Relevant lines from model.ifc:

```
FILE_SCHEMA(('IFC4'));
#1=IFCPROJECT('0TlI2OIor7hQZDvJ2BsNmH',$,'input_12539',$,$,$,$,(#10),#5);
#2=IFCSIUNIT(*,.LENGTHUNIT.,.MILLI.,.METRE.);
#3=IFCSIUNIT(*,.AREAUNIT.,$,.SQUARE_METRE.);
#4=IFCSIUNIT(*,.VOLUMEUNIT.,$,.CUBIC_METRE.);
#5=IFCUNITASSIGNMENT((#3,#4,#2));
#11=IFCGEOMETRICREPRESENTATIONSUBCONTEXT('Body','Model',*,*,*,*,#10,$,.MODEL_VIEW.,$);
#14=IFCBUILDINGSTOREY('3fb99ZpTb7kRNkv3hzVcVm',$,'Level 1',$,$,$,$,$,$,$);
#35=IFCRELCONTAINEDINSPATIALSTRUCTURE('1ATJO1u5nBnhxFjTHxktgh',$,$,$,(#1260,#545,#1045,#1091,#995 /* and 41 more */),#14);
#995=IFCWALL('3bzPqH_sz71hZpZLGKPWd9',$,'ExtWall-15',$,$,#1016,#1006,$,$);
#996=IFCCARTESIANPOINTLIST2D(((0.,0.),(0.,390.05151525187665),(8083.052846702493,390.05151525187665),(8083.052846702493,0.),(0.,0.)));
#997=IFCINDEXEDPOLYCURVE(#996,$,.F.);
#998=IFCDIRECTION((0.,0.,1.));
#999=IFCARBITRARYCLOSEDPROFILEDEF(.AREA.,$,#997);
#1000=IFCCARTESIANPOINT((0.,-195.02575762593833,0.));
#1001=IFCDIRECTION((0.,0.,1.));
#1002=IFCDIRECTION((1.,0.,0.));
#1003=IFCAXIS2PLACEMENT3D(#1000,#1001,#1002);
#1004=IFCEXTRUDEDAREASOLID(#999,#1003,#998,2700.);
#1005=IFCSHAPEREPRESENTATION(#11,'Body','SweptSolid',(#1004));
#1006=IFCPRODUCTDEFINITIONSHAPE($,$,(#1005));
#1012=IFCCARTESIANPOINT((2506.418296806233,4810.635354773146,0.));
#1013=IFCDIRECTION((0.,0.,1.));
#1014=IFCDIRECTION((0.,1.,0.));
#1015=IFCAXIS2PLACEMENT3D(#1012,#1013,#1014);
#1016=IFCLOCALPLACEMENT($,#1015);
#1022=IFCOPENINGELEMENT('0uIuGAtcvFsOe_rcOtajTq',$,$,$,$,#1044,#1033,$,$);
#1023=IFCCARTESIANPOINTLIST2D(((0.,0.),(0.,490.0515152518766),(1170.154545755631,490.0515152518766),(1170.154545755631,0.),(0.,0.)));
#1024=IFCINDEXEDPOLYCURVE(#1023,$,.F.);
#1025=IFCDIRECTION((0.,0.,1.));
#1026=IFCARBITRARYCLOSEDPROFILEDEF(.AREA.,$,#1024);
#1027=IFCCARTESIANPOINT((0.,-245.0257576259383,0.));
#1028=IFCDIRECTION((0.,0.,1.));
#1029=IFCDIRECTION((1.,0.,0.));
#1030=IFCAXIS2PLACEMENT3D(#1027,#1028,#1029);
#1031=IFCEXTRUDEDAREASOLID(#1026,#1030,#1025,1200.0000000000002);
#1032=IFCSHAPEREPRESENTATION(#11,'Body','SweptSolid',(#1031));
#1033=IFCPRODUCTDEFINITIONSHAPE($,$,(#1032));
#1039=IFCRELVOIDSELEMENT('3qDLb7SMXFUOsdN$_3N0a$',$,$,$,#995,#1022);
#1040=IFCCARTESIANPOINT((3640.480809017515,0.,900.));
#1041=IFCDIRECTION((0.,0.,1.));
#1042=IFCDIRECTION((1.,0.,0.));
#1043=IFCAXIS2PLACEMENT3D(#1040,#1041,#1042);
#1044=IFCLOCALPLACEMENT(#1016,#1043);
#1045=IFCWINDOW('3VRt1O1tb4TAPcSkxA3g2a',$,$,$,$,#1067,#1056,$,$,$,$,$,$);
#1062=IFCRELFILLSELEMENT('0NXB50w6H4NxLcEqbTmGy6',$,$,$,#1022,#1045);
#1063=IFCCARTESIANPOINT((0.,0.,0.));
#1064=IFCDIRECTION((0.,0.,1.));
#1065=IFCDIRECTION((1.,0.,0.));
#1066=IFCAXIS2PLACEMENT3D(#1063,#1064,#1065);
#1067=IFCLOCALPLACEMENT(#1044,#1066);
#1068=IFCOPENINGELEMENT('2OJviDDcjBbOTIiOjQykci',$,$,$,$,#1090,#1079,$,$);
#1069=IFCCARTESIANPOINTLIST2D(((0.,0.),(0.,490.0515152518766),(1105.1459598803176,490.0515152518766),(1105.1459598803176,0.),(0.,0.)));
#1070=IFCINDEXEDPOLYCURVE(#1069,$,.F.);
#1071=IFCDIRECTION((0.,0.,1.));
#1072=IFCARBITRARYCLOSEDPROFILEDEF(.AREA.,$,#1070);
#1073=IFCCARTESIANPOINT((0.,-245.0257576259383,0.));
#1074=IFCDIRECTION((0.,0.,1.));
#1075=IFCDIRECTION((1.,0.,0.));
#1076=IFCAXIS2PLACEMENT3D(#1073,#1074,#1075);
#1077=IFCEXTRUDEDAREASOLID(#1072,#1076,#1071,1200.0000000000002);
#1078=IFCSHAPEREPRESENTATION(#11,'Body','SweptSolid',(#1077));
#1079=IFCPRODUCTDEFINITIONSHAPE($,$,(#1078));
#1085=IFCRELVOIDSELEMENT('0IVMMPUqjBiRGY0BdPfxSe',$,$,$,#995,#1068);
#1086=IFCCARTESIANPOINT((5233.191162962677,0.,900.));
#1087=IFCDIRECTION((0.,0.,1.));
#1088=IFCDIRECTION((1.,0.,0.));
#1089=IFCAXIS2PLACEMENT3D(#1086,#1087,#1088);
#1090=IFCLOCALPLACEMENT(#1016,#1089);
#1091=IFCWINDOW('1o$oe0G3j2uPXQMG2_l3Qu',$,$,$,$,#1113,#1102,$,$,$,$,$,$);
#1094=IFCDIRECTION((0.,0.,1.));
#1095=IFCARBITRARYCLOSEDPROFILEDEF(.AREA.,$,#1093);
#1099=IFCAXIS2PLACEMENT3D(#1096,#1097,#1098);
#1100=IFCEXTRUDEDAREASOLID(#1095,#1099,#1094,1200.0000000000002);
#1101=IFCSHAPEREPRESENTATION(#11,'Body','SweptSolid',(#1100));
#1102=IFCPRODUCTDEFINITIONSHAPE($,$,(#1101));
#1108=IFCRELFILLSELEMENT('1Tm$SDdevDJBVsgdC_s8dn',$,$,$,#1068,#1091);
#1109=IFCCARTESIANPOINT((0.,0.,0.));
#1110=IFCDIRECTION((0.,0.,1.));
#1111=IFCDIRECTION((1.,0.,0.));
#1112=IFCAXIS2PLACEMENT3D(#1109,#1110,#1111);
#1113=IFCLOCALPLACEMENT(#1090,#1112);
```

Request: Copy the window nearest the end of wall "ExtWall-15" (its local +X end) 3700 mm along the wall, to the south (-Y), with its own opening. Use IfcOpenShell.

```python
import ifcopenshell
import ifcopenshell.api.feature
import ifcopenshell.api.geometry
import ifcopenshell.api.root
import ifcopenshell.geom
import ifcopenshell.util.element
import ifcopenshell.util.placement
import ifcopenshell.util.shape

model = ifcopenshell.open("model.ifc")
settings = ifcopenshell.geom.settings()


def volume(element):
    """Net volume in cubic metres, openings subtracted."""
    shape = ifcopenshell.geom.create_shape(settings, element)
    return ifcopenshell.util.shape.get_volume(shape.geometry)


window = model.by_guid("1o$oe0G3j2uPXQMG2_l3Qu")
opening = window.FillsVoids[0].RelatingOpeningElement
wall = opening.VoidsElements[0].RelatingBuildingElement
before = volume(wall)
shift = ifcopenshell.util.placement.get_local_placement(wall.ObjectPlacement)[:3, 0] * -3700.0

# copy_class copies the void relationship, type, container and properties, but no geometry.
new_opening = ifcopenshell.api.root.copy_class(model, product=opening)
new_opening.Representation = ifcopenshell.util.element.copy_deep(
    model, opening.Representation, exclude=["IfcGeometricRepresentationContext", "IfcRepresentationMap"]
)
new_window = ifcopenshell.api.root.copy_class(model, product=window)
new_window.Representation = ifcopenshell.util.element.copy_deep(
    model, window.Representation, exclude=["IfcGeometricRepresentationContext", "IfcRepresentationMap"]
)
ifcopenshell.api.feature.add_filling(model, opening=new_opening, element=new_window)

for old, new in ((opening, new_opening), (window, new_window)):
    matrix = ifcopenshell.util.placement.get_local_placement(old.ObjectPlacement)
    matrix[:3, 3] += shift
    ifcopenshell.api.geometry.edit_object_placement(model, product=new, matrix=matrix, is_si=False)

after = volume(wall)

print(f"wall volume {before:.3f} -> {after:.3f} m3")

model.write("model_rev.ifc")
```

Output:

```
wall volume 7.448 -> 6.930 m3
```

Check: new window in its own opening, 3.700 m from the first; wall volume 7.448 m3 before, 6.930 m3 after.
